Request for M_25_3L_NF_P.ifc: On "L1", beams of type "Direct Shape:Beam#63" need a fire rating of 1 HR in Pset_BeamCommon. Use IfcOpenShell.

First a look at what the model holds.

```python
import ifcopenshell
import ifcopenshell.util.element

model = ifcopenshell.open("M_25_3L_NF_P.ifc")
print(model.schema)
storey = next(s for s in model.by_type("IfcBuildingStorey") if s.Name == "L1")
beams = [e for e in ifcopenshell.util.element.get_decomposition(storey) if e.is_a("IfcBeam")]
seen = {}
for e in beams:
    element_type = ifcopenshell.util.element.get_type(e)
    key = (element_type.Name if element_type != e and element_type else None, ifcopenshell.util.element.get_pset(e, "Pset_BeamCommon", "FireRating"))
    seen[key] = seen.get(key, 0) + 1
for (name, value), count in sorted(seen.items(), key=str):
    print(count, "x", name, "|", value)
```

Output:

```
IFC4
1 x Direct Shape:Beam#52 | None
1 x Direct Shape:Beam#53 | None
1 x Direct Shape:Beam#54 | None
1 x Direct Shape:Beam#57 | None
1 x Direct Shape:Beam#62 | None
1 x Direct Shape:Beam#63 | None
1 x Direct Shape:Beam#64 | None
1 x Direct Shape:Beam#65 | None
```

```python
import ifcopenshell
import ifcopenshell.api.pset
import ifcopenshell.util.element

model = ifcopenshell.open("M_25_3L_NF_P.ifc")

storey = next(s for s in model.by_type("IfcBuildingStorey") if s.Name == "L1")
beams = [e for e in ifcopenshell.util.element.get_decomposition(storey) if e.is_a("IfcBeam")]

count = 0
for e in beams:
    element_type = ifcopenshell.util.element.get_type(e)
    if element_type in (None, e) or element_type.Name != "Direct Shape:Beam#63":
        continue
    # add_pset returns the element's existing set when there is one.
    pset = ifcopenshell.api.pset.add_pset(model, product=e, name="Pset_BeamCommon")
    ifcopenshell.api.pset.edit_pset(model, pset=pset, properties={"FireRating": "1 HR"})
    count += 1

print(count, "beams updated")

model.write("M_25_3L_NF_P_v2.ifc")
```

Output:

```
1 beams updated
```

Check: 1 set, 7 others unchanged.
